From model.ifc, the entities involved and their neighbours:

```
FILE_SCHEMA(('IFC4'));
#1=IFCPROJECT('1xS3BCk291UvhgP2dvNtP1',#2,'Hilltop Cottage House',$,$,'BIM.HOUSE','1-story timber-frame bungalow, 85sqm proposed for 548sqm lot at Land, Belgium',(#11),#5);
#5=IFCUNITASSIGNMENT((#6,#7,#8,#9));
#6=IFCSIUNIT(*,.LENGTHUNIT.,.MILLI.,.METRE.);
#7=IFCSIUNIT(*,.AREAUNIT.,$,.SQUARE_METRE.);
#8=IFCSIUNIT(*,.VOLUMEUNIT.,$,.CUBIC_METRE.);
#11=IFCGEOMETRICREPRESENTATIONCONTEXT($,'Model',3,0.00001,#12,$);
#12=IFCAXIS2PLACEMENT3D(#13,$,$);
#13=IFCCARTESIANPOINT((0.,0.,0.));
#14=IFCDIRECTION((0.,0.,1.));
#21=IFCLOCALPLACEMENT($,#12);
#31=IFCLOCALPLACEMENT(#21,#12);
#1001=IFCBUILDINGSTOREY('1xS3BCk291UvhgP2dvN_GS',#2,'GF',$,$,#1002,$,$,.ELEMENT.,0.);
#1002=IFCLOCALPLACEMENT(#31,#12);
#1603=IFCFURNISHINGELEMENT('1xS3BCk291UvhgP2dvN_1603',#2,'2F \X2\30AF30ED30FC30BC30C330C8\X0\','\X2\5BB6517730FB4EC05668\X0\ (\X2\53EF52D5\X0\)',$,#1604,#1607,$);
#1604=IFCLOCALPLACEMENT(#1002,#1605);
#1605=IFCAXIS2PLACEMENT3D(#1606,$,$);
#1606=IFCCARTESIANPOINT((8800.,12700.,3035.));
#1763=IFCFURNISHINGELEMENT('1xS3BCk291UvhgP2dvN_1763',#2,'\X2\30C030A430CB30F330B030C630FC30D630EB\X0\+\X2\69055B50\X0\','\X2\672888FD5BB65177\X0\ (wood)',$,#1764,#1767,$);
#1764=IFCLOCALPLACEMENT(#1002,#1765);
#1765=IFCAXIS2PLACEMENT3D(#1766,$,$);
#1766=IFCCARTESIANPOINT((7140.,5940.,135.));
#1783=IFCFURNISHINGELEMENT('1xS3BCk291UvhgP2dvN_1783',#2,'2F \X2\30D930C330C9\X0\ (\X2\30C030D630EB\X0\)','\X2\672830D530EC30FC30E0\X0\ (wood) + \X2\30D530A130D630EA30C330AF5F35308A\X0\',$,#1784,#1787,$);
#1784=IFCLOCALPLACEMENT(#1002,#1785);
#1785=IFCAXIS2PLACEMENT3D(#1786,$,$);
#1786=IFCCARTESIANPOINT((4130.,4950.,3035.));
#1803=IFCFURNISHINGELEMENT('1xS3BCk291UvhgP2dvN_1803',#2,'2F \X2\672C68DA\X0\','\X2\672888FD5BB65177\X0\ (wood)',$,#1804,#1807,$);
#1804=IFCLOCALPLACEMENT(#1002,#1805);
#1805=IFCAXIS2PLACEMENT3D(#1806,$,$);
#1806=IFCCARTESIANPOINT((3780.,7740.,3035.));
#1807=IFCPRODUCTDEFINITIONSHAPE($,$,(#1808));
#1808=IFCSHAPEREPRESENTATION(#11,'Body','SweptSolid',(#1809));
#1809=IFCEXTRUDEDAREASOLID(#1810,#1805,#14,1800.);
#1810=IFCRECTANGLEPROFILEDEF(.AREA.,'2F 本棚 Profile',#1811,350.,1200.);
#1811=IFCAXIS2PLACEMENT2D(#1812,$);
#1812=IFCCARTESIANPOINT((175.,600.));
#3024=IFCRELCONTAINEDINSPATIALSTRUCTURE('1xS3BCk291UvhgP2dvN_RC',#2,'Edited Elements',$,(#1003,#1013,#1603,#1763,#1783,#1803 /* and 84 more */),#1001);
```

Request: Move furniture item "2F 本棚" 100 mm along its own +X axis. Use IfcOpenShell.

```python
import ifcopenshell
import ifcopenshell.api.geometry
import ifcopenshell.util.placement
import ifcopenshell.util.unit

model = ifcopenshell.open("model.ifc")
unit_scale = ifcopenshell.util.unit.calculate_unit_scale(model)

item = model.by_guid("1xS3BCk291UvhgP2dvN_1803")
matrix = ifcopenshell.util.placement.get_local_placement(item.ObjectPlacement)
matrix[:3, 3] += matrix[:3, 0] * 0.1 / unit_scale
ifcopenshell.api.geometry.edit_object_placement(model, product=item, matrix=matrix, is_si=False)

print(ifcopenshell.util.placement.get_local_placement(item.ObjectPlacement).round(3) + 0.0)

model.write("model_rev.ifc")
```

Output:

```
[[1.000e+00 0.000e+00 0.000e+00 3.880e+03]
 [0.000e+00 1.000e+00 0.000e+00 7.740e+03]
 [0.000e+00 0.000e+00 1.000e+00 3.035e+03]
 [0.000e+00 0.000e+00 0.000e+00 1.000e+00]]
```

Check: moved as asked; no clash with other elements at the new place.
